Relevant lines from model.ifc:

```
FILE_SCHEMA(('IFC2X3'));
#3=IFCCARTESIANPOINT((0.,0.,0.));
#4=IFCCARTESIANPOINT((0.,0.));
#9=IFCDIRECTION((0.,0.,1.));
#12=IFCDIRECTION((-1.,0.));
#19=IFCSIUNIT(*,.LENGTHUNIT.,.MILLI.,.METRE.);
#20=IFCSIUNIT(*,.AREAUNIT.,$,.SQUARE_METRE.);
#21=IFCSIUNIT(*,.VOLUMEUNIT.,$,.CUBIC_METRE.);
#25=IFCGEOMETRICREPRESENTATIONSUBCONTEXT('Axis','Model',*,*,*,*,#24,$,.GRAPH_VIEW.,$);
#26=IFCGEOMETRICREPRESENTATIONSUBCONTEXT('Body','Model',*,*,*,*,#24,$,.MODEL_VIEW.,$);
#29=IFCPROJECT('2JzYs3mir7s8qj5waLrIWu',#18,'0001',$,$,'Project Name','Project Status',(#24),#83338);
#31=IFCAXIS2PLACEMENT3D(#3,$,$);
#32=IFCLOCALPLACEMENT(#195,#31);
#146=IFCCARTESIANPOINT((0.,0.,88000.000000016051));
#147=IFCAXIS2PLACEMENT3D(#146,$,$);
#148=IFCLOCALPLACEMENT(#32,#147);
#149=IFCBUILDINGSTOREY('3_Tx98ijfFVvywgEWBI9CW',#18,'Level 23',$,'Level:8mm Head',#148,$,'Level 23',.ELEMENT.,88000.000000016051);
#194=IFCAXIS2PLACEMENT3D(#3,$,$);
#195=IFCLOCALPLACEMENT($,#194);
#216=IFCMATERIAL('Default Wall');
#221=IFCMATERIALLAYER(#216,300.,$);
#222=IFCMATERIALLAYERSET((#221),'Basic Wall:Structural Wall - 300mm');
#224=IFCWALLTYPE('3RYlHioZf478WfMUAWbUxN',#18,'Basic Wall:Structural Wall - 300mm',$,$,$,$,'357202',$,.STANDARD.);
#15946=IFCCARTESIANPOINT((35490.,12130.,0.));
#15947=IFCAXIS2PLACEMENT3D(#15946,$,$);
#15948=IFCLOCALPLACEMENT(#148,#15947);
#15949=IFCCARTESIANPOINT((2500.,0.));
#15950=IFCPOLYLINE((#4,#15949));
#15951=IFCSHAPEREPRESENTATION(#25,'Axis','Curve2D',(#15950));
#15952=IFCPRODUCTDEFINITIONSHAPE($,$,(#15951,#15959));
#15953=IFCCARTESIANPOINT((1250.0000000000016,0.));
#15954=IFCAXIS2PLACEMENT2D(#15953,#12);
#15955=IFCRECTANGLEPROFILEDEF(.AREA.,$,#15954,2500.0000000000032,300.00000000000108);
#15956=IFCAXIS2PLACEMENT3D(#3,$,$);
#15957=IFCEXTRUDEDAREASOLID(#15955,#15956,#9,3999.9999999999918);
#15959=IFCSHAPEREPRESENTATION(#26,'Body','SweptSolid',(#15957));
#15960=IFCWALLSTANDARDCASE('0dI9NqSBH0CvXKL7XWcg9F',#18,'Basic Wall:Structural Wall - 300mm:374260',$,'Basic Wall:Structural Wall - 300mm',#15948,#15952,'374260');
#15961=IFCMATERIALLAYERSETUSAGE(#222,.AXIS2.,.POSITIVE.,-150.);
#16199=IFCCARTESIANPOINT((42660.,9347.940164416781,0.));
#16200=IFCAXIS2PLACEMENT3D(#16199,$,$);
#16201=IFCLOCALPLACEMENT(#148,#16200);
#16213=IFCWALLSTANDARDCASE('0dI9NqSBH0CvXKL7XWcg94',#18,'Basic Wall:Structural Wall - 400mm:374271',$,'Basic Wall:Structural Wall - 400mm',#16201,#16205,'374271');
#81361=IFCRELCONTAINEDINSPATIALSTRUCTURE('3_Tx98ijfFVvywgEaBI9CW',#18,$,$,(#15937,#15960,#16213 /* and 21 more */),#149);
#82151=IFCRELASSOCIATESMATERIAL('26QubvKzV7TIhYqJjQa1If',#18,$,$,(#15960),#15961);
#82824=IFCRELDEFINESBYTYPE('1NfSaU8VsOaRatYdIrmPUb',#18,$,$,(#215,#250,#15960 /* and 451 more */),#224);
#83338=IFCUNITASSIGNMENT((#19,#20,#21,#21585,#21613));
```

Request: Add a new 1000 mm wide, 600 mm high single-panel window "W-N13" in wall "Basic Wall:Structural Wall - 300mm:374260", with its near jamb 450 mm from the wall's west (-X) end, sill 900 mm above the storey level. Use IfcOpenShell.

```python
import numpy as np
import ifcopenshell
import ifcopenshell.api.feature
import ifcopenshell.api.geometry
import ifcopenshell.api.root
import ifcopenshell.api.spatial
import ifcopenshell.api.type
import ifcopenshell.geom
import ifcopenshell.util.element
import ifcopenshell.util.placement
import ifcopenshell.util.representation
import ifcopenshell.util.shape
import ifcopenshell.util.unit

model = ifcopenshell.open("model.ifc")
unit_scale = ifcopenshell.util.unit.calculate_unit_scale(model)
settings = ifcopenshell.geom.settings()


def volume(element):
    """Net volume in cubic metres, openings subtracted."""
    shape = ifcopenshell.geom.create_shape(settings, element)
    return ifcopenshell.util.shape.get_volume(shape.geometry)


wall = model.by_guid("0dI9NqSBH0CvXKL7XWcg9F")
storey = ifcopenshell.util.element.get_container(wall, ifc_class="IfcBuildingStorey")
context = ifcopenshell.util.representation.get_context(model, "Model", "Body", "MODEL_VIEW")
before = volume(wall)

width, height, from_end, sill = 1, 0.6, 0.45, 0.9  # metres

# The wall runs along its own X axis, and the end named is its -X end.
wall_shape = ifcopenshell.geom.create_shape(settings, wall)
x, y, z = ifcopenshell.util.shape.get_vertices(wall_shape.geometry).T
start = x.min() + from_end
face, thickness = float(y.min()), float(y.max() - y.min())
wall_matrix = ifcopenshell.util.placement.get_local_placement(wall.ObjectPlacement)
level = ifcopenshell.util.placement.get_local_placement(storey.ObjectPlacement)[2, 3]


def in_wall(x, y):
    """Placement at x, y metres in the wall's axes, at sill height."""
    matrix = wall_matrix.copy()
    matrix[:, 3] = wall_matrix @ np.array([x / unit_scale, y / unit_scale, 0.0, 1.0])
    matrix[2, 3] = level + sill / unit_scale
    return matrix


# Opening: a box that overshoots both wall faces by 50 mm.
opening = ifcopenshell.api.root.create_entity(model, ifc_class="IfcOpeningElement")
box = ifcopenshell.api.geometry.add_wall_representation(
    model, context=context, length=width, height=height, thickness=thickness + 0.1
)
ifcopenshell.api.geometry.assign_representation(model, product=opening, representation=box)
ifcopenshell.api.geometry.edit_object_placement(model, product=opening, matrix=in_wall(start, face - 0.05), is_si=False)
ifcopenshell.api.feature.add_feature(model, feature=opening, element=wall)

window = ifcopenshell.api.root.create_entity(model, ifc_class="IfcWindow", name="W-N13")
window.OverallWidth, window.OverallHeight = width / unit_scale, height / unit_scale
body = ifcopenshell.api.geometry.add_window_representation(
    model,
    context=context,
    overall_width=window.OverallWidth,
    overall_height=window.OverallHeight,
    partition_type="SINGLE_PANEL",
)
ifcopenshell.api.geometry.assign_representation(model, product=window, representation=body)
ifcopenshell.api.spatial.assign_container(model, products=[window], relating_structure=storey)
fills = ifcopenshell.api.feature.add_filling(model, opening=opening, element=window)
fills.OwnerHistory = window.OwnerHistory  # required in IFC2X3

# IFC2X3 keeps the operation on the window style.
style = ifcopenshell.api.root.create_entity(model, ifc_class="IfcWindowStyle", name="W-N13")
style.OperationType, style.ConstructionType = "SINGLE_PANEL", "NOTDEFINED"
style.ParameterTakesPrecedence = style.Sizeable = False
ifcopenshell.api.type.assign_type(model, related_objects=[window], relating_type=style)

# Centre the window in the wall's thickness.
ifcopenshell.api.geometry.edit_object_placement(model, product=window, matrix=in_wall(start, face), is_si=False)
window_shape = ifcopenshell.geom.create_shape(settings, window)
depth = ifcopenshell.util.shape.get_vertices(window_shape.geometry)[:, 1]
offset = face + thickness / 2 - (depth.min() + depth.max()) / 2
ifcopenshell.api.geometry.edit_object_placement(model, product=window, matrix=in_wall(start, offset), is_si=False)

after = volume(wall)

print(f"wall volume {before:.3f} -> {after:.3f} m3")

model.write("model_rev.ifc")
```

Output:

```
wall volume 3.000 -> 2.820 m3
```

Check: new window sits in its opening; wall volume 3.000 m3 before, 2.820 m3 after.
